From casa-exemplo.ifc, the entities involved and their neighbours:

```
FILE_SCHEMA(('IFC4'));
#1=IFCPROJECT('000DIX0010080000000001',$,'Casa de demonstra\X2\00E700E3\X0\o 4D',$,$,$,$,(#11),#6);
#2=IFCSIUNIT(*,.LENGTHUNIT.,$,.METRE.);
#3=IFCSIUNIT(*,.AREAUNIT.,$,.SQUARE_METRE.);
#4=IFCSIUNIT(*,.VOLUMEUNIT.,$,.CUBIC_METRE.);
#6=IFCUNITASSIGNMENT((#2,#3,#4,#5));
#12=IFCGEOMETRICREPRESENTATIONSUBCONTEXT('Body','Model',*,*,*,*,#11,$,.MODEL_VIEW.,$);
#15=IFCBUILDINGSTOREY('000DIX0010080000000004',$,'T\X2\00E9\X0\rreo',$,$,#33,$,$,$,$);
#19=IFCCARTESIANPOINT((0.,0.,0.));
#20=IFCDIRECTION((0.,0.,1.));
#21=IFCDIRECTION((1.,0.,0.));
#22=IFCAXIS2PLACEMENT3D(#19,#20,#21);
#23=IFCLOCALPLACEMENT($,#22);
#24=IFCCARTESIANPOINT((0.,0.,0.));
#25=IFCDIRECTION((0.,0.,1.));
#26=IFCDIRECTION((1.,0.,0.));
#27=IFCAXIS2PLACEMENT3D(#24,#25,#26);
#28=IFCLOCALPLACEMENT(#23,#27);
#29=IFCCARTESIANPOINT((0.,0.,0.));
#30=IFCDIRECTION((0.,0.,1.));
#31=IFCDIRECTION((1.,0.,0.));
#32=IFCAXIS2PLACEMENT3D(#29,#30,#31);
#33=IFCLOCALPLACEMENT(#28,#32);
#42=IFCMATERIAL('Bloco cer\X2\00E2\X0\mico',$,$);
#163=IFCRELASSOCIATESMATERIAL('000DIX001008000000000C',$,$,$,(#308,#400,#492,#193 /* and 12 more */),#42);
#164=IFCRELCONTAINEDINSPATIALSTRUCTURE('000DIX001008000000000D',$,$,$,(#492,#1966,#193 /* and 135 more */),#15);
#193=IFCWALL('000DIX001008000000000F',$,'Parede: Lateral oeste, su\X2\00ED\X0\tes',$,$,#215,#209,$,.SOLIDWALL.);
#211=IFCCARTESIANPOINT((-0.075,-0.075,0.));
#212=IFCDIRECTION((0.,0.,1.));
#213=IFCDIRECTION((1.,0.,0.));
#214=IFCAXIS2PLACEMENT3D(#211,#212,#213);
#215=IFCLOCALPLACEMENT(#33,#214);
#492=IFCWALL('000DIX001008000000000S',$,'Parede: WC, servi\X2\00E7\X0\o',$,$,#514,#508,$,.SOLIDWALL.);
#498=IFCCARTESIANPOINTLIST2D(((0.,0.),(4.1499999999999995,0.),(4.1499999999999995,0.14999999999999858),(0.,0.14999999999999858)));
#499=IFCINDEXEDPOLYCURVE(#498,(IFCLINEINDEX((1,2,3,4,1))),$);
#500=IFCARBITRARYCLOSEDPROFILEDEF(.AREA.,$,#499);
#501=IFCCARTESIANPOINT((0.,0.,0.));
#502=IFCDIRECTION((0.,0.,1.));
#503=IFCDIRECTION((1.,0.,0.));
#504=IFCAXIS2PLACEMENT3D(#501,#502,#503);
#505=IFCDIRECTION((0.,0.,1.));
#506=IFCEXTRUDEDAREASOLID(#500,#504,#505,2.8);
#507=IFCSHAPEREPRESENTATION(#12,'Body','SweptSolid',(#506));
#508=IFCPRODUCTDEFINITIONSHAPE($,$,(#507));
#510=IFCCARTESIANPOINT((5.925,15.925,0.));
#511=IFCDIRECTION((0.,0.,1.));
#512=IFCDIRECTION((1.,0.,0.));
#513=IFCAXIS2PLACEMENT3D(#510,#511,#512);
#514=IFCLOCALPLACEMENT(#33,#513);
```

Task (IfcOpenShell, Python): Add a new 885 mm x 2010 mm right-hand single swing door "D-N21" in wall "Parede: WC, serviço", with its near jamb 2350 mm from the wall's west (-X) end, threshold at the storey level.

```python
import numpy as np
import ifcopenshell
import ifcopenshell.api.feature
import ifcopenshell.api.geometry
import ifcopenshell.api.root
import ifcopenshell.api.spatial
import ifcopenshell.geom
import ifcopenshell.util.element
import ifcopenshell.util.placement
import ifcopenshell.util.representation
import ifcopenshell.util.shape
import ifcopenshell.util.unit

model = ifcopenshell.open("casa-exemplo.ifc")
unit_scale = ifcopenshell.util.unit.calculate_unit_scale(model)
settings = ifcopenshell.geom.settings()


def volume(element):
    """Net volume in cubic metres, openings subtracted."""
    shape = ifcopenshell.geom.create_shape(settings, element)
    return ifcopenshell.util.shape.get_volume(shape.geometry)


wall = model.by_guid("000DIX001008000000000S")
storey = ifcopenshell.util.element.get_container(wall, ifc_class="IfcBuildingStorey")
context = ifcopenshell.util.representation.get_context(model, "Model", "Body", "MODEL_VIEW")
before = volume(wall)

width, height, from_end, sill = 0.885, 2.01, 2.35, 0.0  # metres

# The wall runs along its own X axis, and the end named is its -X end.
wall_shape = ifcopenshell.geom.create_shape(settings, wall)
x, y, z = ifcopenshell.util.shape.get_vertices(wall_shape.geometry).T
start = x.min() + from_end
face, thickness = float(y.min()), float(y.max() - y.min())
wall_matrix = ifcopenshell.util.placement.get_local_placement(wall.ObjectPlacement)
level = ifcopenshell.util.placement.get_local_placement(storey.ObjectPlacement)[2, 3]


def in_wall(x, y):
    """Placement at x, y metres in the wall's axes, at sill height."""
    matrix = wall_matrix.copy()
    matrix[:, 3] = wall_matrix @ np.array([x / unit_scale, y / unit_scale, 0.0, 1.0])
    matrix[2, 3] = level + sill / unit_scale
    return matrix


# Opening: a box that overshoots both wall faces by 50 mm.
opening = ifcopenshell.api.root.create_entity(model, ifc_class="IfcOpeningElement", predefined_type="OPENING")
box = ifcopenshell.api.geometry.add_wall_representation(
    model, context=context, length=width, height=height, thickness=thickness + 0.1
)
ifcopenshell.api.geometry.assign_representation(model, product=opening, representation=box)
ifcopenshell.api.geometry.edit_object_placement(model, product=opening, matrix=in_wall(start, face - 0.05), is_si=False)
ifcopenshell.api.feature.add_feature(model, feature=opening, element=wall)

door = ifcopenshell.api.root.create_entity(model, ifc_class="IfcDoor", name="D-N21", predefined_type="DOOR")
door.OverallWidth, door.OverallHeight = width / unit_scale, height / unit_scale
door.OperationType = "SINGLE_SWING_RIGHT"
body = ifcopenshell.api.geometry.add_door_representation(
    model,
    context=context,
    overall_width=door.OverallWidth,
    overall_height=door.OverallHeight,
    operation_type="SINGLE_SWING_RIGHT",
    lining_properties={"LiningDepth": thickness / unit_scale, "ThresholdDepth": thickness / unit_scale},
)
ifcopenshell.api.geometry.assign_representation(model, product=door, representation=body)
ifcopenshell.api.spatial.assign_container(model, products=[door], relating_structure=storey)
ifcopenshell.api.feature.add_filling(model, opening=opening, element=door)

# The lining spans the wall, so the door starts at the wall face.
ifcopenshell.api.geometry.edit_object_placement(model, product=door, matrix=in_wall(start, face), is_si=False)

after = volume(wall)

print(f"wall volume {before:.3f} -> {after:.3f} m3")

model.write("casa-exemplo-out.ifc")
```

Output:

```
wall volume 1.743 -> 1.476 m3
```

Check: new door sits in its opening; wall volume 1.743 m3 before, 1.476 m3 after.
